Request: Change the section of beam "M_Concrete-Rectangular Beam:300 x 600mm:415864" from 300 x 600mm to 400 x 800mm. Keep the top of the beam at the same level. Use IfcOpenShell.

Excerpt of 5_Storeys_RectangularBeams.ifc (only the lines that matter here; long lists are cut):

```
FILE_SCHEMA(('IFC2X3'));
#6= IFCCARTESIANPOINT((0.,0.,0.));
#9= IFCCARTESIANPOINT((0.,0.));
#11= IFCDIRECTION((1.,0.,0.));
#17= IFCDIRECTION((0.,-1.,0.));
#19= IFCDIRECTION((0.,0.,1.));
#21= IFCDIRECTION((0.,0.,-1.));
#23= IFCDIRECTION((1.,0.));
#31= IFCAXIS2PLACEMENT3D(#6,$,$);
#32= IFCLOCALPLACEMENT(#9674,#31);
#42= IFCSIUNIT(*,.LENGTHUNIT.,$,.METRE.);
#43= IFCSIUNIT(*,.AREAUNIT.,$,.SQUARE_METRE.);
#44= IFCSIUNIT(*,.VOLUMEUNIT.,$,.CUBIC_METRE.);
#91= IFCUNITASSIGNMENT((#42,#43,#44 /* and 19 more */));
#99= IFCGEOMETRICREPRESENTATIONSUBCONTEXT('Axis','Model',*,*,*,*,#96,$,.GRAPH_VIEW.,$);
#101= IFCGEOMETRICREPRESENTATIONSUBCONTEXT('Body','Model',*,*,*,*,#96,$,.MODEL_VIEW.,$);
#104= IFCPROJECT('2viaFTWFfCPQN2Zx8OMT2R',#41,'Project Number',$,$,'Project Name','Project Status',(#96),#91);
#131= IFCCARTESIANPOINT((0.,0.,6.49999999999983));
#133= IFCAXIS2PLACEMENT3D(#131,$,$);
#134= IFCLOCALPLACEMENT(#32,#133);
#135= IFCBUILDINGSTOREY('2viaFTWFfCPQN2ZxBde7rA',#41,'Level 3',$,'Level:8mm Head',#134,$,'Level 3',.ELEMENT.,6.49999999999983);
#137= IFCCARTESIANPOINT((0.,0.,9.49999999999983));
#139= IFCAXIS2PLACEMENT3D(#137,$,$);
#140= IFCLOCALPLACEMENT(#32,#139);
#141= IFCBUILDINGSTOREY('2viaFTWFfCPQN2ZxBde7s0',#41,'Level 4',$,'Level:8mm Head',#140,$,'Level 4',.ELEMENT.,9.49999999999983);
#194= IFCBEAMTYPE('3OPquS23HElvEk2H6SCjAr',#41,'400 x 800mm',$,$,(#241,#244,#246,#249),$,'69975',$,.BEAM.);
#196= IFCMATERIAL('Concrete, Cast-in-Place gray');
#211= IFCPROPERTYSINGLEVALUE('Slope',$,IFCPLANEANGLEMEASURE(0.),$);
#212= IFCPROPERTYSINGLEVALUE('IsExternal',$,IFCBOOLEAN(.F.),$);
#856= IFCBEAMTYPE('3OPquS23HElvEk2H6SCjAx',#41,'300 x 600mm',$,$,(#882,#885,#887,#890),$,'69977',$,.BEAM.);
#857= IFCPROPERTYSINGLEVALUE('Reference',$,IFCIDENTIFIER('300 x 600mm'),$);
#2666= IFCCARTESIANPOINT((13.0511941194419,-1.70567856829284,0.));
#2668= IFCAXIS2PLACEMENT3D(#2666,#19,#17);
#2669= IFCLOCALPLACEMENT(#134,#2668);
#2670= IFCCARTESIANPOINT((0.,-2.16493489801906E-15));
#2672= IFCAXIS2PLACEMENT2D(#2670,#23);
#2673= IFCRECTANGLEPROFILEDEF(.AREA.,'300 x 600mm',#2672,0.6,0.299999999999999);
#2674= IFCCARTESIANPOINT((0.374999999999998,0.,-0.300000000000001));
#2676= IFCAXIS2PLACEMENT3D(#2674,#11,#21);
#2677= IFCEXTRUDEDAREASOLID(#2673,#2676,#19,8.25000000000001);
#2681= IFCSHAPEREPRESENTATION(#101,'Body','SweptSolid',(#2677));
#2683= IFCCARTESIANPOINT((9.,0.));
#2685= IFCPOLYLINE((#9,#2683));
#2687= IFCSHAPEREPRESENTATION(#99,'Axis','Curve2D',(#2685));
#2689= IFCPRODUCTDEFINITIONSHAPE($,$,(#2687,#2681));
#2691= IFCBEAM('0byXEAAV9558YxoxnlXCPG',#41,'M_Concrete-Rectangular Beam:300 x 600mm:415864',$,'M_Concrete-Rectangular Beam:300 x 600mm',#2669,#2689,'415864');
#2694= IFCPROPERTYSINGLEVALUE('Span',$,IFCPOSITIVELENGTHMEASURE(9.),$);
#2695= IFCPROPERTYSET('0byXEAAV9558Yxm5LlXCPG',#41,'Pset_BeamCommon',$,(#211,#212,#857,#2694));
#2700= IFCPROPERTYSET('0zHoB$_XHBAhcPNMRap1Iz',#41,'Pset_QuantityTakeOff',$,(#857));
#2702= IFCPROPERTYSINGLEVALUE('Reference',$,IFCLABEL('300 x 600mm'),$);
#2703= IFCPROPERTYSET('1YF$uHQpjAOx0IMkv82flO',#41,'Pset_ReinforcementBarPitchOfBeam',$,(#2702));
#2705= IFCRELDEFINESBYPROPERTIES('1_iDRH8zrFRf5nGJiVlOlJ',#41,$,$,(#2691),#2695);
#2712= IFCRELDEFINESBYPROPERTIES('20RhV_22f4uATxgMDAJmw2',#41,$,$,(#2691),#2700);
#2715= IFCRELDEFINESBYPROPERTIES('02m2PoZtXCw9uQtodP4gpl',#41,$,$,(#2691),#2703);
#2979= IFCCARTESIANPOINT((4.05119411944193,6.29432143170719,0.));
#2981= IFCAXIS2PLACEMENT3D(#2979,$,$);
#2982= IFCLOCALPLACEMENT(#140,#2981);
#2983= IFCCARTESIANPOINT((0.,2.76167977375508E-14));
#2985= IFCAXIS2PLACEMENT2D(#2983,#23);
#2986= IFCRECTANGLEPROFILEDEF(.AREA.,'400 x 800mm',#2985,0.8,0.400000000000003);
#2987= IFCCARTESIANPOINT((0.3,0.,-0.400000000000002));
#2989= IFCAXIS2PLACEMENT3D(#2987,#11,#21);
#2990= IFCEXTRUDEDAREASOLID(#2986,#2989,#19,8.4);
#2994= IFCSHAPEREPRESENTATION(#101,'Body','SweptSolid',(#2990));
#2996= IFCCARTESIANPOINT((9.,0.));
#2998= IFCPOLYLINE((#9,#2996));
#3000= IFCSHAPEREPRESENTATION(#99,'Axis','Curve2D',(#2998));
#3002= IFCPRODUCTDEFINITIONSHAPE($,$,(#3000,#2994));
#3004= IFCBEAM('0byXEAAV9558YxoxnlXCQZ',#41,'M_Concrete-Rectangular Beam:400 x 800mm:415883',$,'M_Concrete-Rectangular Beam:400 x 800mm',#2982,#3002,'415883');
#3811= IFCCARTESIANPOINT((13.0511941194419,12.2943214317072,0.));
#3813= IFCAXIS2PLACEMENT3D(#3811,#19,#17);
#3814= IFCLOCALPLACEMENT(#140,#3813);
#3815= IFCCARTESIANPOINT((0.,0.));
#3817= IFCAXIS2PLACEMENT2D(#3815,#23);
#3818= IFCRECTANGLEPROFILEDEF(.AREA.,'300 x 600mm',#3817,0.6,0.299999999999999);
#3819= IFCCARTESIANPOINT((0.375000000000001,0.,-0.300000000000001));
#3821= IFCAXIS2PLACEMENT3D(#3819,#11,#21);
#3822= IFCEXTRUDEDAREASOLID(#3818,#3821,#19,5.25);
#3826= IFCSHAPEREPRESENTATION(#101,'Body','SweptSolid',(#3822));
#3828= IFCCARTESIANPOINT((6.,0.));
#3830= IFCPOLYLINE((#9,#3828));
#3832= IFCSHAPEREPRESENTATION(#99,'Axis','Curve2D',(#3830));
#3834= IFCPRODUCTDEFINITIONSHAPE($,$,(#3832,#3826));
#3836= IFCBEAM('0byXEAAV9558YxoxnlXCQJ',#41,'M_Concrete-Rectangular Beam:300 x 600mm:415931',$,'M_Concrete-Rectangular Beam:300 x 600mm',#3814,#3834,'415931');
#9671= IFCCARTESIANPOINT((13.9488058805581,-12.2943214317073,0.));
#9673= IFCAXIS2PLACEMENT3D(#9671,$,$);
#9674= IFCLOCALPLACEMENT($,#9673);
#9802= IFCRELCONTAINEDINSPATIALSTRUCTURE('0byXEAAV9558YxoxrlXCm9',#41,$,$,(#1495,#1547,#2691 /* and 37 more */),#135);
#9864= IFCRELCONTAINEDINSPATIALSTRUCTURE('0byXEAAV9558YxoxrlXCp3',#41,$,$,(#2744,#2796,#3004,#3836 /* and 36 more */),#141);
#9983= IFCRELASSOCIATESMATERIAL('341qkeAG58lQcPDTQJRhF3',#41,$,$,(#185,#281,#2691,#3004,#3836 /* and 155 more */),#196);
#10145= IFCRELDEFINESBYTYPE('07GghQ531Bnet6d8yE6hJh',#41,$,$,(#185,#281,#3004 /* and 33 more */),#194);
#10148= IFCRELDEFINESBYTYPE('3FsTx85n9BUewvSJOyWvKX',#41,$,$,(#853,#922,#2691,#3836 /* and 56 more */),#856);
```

```python
import ifcopenshell
import ifcopenshell.api.pset
import ifcopenshell.api.type
import ifcopenshell.util.element
import ifcopenshell.util.representation

model = ifcopenshell.open("5_Storeys_RectangularBeams.ifc")

member = model.by_guid("0byXEAAV9558YxoxnlXCPG")
source = next(p for p in model.by_type("IfcRectangleProfileDef") if p.ProfileName == "400 x 800mm")

body = ifcopenshell.util.representation.get_representation(member, "Model", "Body")
solid = body.Items[0]
old_profile = solid.SweptArea

# Copy the section's sizes but keep this member's own profile position.
profile = ifcopenshell.util.element.copy(model, source)
# Profiles are centred, so shift by half the change in depth to hold the top.
shift = (old_profile.XDim - profile.XDim) / 2
x, y = old_profile.Position.Location.Coordinates
up = (-1.0, 0.0)  # upwards, in the solid's own plane
location = model.createIfcCartesianPoint((x + up[0] * shift, y + up[1] * shift))
profile.Position = model.createIfcAxis2Placement2D(location, old_profile.Position.RefDirection)
solid.SweptArea = profile
if not model.get_total_inverses(old_profile):
    ifcopenshell.util.element.remove_deep2(model, old_profile)

new_type = model.by_guid("3OPquS23HElvEk2H6SCjAr")
ifcopenshell.api.type.assign_type(
    model, related_objects=[member], relating_type=new_type, should_map_representations=False
)
member.Name = member.Name.replace("300 x 600mm", "400 x 800mm")
member.ObjectType = "M_Concrete-Rectangular Beam:400 x 800mm"
pset = model.by_id(ifcopenshell.util.element.get_pset(member, "Pset_BeamCommon", should_inherit=False)["id"])
ifcopenshell.api.pset.edit_pset(model, pset=pset, properties={"Reference": "400 x 800mm"})
pset = model.by_id(ifcopenshell.util.element.get_pset(member, "Pset_QuantityTakeOff", should_inherit=False)["id"])
ifcopenshell.api.pset.edit_pset(model, pset=pset, properties={"Reference": "400 x 800mm"})
pset = model.by_id(ifcopenshell.util.element.get_pset(member, "Pset_ReinforcementBarPitchOfBeam", should_inherit=False)["id"])
ifcopenshell.api.pset.edit_pset(model, pset=pset, properties={"Reference": "400 x 800mm"})

print(solid.SweptArea)

model.write("5_Storeys_RectangularBeams_edited.ifc")
```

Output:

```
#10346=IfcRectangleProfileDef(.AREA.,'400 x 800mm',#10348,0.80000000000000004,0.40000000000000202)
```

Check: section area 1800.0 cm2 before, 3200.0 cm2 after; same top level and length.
